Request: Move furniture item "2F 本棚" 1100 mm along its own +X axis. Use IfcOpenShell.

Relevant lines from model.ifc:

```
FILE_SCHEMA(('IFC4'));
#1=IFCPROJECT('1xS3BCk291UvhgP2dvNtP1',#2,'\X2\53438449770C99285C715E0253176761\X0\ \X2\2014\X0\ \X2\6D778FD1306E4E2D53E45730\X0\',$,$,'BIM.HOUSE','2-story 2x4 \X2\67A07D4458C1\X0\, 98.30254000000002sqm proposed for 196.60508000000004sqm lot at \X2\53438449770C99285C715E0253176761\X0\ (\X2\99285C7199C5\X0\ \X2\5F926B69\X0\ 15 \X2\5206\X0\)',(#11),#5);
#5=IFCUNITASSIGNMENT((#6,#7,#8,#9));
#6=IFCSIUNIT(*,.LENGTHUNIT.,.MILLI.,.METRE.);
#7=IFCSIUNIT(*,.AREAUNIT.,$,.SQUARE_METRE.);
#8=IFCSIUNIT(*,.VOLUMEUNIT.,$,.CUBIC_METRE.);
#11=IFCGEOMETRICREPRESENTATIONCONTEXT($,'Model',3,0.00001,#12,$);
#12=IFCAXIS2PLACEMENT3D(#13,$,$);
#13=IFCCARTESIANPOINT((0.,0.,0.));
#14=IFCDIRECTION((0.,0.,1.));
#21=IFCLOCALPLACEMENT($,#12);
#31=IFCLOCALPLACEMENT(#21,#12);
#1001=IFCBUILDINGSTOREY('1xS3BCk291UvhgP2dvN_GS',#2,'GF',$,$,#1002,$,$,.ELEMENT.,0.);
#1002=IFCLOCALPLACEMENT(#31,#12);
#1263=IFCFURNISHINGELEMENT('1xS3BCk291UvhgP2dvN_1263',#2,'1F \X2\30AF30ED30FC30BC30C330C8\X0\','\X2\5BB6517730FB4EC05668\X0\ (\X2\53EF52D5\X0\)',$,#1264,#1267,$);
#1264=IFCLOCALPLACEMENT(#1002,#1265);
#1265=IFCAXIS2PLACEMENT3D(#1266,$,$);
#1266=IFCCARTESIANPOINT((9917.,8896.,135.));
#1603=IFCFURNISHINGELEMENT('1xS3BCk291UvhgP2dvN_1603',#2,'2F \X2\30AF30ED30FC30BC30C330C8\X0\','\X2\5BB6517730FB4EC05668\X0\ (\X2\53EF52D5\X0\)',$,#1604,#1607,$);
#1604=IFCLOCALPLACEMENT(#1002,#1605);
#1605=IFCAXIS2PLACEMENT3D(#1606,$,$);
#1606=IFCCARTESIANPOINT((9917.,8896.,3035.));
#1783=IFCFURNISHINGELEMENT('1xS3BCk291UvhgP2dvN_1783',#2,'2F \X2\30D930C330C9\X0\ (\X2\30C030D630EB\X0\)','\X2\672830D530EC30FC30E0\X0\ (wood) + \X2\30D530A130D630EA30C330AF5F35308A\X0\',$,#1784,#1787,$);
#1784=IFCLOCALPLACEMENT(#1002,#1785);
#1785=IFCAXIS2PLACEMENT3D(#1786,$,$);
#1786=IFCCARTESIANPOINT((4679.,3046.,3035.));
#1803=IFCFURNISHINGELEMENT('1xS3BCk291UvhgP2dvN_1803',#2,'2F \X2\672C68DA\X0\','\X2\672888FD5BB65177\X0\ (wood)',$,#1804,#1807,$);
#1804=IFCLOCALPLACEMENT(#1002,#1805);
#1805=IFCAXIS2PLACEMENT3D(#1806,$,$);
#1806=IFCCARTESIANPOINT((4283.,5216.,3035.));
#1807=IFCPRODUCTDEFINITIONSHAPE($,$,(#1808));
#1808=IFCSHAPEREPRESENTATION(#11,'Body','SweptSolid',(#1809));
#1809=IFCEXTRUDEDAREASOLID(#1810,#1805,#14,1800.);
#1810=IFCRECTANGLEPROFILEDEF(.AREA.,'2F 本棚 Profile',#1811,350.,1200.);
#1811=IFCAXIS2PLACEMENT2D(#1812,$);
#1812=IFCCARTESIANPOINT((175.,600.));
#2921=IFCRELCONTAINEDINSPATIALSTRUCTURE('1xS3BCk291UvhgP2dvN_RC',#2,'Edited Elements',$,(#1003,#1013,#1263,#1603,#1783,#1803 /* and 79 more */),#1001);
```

```python
import ifcopenshell
import ifcopenshell.api.geometry
import ifcopenshell.util.placement

model = ifcopenshell.open("model.ifc")

item = model.by_guid("1xS3BCk291UvhgP2dvN_1803")
matrix = ifcopenshell.util.placement.get_local_placement(item.ObjectPlacement)
matrix[:3, 3] += matrix[:3, 0] * 1100.0
ifcopenshell.api.geometry.edit_object_placement(model, product=item, matrix=matrix, is_si=False)

print(ifcopenshell.util.placement.get_local_placement(item.ObjectPlacement).round(3) + 0.0)

model.write("model_updated.ifc")
```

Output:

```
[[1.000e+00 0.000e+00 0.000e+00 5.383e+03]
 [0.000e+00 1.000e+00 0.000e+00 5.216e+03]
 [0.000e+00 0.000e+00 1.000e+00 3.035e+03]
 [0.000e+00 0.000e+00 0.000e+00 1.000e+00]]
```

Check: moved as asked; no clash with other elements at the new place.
